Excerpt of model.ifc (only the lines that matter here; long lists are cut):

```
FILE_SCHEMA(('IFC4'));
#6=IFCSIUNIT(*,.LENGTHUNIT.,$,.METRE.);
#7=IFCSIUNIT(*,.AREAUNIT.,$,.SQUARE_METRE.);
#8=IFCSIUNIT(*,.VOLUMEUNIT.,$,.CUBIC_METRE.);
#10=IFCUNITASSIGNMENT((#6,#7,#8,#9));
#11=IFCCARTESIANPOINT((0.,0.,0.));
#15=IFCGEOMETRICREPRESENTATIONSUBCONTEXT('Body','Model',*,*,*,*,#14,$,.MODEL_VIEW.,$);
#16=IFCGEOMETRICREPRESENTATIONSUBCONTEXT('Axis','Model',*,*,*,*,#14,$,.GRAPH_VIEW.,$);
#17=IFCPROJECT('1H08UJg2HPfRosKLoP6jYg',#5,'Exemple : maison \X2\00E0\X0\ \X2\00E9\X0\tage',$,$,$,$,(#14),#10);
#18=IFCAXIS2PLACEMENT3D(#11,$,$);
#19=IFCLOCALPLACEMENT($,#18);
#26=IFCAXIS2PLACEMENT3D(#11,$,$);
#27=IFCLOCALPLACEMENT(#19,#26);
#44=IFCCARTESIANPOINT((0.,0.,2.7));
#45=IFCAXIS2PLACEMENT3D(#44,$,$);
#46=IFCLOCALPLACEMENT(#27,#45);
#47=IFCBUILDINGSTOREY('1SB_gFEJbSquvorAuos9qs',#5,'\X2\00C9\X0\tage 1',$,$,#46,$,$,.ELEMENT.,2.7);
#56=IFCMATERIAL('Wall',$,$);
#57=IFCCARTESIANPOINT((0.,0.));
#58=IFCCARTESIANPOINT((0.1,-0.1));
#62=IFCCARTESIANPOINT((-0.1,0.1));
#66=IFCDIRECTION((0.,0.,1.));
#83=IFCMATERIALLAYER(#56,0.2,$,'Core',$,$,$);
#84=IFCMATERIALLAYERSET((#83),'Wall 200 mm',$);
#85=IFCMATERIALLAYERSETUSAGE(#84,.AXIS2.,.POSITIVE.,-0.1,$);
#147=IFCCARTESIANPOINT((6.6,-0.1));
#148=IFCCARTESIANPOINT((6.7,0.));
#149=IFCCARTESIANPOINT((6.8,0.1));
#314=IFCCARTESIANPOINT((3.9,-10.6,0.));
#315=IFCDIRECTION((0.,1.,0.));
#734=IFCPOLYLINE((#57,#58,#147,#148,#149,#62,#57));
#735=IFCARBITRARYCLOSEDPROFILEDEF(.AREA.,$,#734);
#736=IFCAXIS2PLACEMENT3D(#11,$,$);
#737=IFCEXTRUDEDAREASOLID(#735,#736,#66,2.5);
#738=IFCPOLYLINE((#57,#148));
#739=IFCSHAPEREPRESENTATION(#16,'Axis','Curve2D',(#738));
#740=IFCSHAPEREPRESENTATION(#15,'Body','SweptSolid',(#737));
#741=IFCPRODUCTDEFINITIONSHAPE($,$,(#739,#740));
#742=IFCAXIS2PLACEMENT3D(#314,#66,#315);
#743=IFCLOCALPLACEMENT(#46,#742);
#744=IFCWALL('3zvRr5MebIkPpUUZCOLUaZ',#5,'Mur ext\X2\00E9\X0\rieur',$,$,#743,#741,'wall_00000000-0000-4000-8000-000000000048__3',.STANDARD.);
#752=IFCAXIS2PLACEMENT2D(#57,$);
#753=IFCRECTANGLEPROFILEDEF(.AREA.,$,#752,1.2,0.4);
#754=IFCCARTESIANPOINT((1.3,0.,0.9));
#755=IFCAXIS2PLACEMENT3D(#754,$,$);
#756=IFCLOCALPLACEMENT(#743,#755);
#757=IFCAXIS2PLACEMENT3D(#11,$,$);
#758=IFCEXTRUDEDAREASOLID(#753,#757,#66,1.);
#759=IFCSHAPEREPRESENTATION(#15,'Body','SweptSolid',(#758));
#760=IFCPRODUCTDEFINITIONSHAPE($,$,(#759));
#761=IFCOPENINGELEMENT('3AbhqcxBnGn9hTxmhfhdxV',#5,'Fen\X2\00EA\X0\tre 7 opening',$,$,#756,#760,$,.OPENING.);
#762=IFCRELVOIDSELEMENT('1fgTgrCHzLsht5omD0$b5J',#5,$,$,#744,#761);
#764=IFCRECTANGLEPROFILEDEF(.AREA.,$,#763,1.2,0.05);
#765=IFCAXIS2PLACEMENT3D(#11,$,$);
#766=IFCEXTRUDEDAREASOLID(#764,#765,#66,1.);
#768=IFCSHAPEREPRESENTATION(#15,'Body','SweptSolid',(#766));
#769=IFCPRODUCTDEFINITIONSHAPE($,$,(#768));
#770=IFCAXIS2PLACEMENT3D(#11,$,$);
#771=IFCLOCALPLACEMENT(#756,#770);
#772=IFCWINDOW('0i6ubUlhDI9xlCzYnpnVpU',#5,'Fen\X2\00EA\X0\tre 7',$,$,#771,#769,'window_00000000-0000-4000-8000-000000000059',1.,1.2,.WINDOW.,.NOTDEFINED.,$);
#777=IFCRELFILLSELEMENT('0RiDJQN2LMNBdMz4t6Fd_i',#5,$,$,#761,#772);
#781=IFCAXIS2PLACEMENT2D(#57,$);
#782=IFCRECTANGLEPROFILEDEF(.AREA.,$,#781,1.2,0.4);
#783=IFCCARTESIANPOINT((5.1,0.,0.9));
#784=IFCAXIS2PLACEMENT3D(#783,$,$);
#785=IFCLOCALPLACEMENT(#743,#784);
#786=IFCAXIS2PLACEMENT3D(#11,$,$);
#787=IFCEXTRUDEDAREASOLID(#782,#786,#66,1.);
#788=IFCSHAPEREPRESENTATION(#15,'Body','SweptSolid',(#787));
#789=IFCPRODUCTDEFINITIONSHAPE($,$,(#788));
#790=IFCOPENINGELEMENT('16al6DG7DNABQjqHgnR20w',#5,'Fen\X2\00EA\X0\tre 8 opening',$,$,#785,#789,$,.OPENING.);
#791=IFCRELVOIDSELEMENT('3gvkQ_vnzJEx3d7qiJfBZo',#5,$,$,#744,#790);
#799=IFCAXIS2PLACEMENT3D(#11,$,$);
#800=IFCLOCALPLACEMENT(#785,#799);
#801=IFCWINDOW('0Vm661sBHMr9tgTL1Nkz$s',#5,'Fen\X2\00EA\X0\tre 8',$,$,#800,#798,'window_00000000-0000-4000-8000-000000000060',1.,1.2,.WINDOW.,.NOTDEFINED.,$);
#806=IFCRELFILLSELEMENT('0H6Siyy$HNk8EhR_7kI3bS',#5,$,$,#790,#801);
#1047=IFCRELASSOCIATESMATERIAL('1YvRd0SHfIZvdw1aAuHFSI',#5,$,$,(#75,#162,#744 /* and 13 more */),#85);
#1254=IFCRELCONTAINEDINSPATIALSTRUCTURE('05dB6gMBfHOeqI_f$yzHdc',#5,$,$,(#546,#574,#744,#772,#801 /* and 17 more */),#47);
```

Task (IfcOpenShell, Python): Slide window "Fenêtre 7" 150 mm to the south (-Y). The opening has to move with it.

```python
import ifcopenshell
import ifcopenshell.api.geometry
import ifcopenshell.util.placement
import ifcopenshell.util.unit

model = ifcopenshell.open("model.ifc")
unit_scale = ifcopenshell.util.unit.calculate_unit_scale(model)

window = model.by_guid("0i6ubUlhDI9xlCzYnpnVpU")
opening = window.FillsVoids[0].RelatingOpeningElement
wall = opening.VoidsElements[0].RelatingBuildingElement

wall_matrix = ifcopenshell.util.placement.get_local_placement(wall.ObjectPlacement)
shift = wall_matrix[:3, 0] * -0.15 / unit_scale
before = ifcopenshell.util.placement.get_local_placement(window.ObjectPlacement)[:3, 3].copy()

# The window is placed relative to its opening, so it follows when the opening moves.
matrix = ifcopenshell.util.placement.get_local_placement(opening.ObjectPlacement)
matrix[:3, 3] += shift
ifcopenshell.api.geometry.edit_object_placement(
    model, product=opening, matrix=matrix, is_si=False, should_transform_children=True
)

after = ifcopenshell.util.placement.get_local_placement(window.ObjectPlacement)[:3, 3]
print("window moved by", (after - before).round(3) + 0.0)

model.write("model_v2.ifc")
```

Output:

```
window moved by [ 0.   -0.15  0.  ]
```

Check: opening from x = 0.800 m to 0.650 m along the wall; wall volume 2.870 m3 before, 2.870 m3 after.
